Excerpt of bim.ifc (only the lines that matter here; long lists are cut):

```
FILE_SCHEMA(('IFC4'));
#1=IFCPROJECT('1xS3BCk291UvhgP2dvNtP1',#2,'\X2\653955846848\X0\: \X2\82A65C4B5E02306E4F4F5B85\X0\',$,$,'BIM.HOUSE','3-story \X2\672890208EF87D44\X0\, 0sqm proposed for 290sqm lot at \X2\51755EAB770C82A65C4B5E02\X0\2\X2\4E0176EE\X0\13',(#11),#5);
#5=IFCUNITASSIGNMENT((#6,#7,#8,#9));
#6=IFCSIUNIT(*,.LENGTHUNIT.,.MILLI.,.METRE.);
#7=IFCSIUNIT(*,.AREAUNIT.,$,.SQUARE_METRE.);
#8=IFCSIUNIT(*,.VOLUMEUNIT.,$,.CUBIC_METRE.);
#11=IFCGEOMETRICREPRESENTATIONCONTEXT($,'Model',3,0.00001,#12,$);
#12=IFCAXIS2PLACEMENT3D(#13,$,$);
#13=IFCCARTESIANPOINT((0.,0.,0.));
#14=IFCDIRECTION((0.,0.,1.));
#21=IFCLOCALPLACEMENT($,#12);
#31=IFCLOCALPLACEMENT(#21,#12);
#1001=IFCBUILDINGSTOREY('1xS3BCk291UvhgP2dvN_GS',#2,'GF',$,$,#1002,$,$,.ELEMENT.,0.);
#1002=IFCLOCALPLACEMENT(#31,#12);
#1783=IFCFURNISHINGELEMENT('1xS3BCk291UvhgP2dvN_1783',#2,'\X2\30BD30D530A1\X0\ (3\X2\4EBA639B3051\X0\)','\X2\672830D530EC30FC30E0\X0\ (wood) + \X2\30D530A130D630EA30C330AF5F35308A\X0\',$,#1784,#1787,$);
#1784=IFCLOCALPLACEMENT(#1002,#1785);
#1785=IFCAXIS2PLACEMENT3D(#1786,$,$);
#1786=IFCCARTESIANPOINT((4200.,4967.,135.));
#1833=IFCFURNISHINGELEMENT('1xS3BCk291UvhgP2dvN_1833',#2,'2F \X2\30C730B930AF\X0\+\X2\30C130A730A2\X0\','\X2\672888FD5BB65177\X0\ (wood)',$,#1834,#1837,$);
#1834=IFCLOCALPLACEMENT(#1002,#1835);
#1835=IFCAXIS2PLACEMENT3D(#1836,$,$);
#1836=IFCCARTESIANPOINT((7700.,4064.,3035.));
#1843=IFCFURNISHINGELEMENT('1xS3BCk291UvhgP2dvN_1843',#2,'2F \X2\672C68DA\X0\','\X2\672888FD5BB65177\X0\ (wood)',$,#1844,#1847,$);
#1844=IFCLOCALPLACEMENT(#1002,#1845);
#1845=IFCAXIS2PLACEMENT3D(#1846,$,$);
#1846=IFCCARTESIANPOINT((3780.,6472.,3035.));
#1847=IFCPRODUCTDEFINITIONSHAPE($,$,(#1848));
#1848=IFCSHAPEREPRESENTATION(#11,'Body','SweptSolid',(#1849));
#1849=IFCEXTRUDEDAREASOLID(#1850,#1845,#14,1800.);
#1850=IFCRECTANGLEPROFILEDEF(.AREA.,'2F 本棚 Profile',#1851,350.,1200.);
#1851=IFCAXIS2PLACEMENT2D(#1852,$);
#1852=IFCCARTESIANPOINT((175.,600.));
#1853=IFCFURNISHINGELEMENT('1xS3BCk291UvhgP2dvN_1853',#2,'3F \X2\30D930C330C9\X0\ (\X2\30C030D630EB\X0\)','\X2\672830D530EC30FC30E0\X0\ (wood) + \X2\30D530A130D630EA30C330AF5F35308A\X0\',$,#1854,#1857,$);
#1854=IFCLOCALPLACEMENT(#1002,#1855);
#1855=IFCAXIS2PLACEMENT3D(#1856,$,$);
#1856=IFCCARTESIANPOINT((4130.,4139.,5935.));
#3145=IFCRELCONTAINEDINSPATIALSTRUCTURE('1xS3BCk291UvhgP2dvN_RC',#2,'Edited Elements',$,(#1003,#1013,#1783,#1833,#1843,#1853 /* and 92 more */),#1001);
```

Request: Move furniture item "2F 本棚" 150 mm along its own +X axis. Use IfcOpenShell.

```python
import ifcopenshell
import ifcopenshell.api.geometry
import ifcopenshell.util.placement

model = ifcopenshell.open("bim.ifc")

item = model.by_id(1843)
matrix = ifcopenshell.util.placement.get_local_placement(item.ObjectPlacement)
matrix[:3, 3] += matrix[:3, 0] * 150.0
ifcopenshell.api.geometry.edit_object_placement(model, product=item, matrix=matrix, is_si=False)

print(ifcopenshell.util.placement.get_local_placement(item.ObjectPlacement).round(3) + 0.0)

model.write("bim_edited.ifc")
```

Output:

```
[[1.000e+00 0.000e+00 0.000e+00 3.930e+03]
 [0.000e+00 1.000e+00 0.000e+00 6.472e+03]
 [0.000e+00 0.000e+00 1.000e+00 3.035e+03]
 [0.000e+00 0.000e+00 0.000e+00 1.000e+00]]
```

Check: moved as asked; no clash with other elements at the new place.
